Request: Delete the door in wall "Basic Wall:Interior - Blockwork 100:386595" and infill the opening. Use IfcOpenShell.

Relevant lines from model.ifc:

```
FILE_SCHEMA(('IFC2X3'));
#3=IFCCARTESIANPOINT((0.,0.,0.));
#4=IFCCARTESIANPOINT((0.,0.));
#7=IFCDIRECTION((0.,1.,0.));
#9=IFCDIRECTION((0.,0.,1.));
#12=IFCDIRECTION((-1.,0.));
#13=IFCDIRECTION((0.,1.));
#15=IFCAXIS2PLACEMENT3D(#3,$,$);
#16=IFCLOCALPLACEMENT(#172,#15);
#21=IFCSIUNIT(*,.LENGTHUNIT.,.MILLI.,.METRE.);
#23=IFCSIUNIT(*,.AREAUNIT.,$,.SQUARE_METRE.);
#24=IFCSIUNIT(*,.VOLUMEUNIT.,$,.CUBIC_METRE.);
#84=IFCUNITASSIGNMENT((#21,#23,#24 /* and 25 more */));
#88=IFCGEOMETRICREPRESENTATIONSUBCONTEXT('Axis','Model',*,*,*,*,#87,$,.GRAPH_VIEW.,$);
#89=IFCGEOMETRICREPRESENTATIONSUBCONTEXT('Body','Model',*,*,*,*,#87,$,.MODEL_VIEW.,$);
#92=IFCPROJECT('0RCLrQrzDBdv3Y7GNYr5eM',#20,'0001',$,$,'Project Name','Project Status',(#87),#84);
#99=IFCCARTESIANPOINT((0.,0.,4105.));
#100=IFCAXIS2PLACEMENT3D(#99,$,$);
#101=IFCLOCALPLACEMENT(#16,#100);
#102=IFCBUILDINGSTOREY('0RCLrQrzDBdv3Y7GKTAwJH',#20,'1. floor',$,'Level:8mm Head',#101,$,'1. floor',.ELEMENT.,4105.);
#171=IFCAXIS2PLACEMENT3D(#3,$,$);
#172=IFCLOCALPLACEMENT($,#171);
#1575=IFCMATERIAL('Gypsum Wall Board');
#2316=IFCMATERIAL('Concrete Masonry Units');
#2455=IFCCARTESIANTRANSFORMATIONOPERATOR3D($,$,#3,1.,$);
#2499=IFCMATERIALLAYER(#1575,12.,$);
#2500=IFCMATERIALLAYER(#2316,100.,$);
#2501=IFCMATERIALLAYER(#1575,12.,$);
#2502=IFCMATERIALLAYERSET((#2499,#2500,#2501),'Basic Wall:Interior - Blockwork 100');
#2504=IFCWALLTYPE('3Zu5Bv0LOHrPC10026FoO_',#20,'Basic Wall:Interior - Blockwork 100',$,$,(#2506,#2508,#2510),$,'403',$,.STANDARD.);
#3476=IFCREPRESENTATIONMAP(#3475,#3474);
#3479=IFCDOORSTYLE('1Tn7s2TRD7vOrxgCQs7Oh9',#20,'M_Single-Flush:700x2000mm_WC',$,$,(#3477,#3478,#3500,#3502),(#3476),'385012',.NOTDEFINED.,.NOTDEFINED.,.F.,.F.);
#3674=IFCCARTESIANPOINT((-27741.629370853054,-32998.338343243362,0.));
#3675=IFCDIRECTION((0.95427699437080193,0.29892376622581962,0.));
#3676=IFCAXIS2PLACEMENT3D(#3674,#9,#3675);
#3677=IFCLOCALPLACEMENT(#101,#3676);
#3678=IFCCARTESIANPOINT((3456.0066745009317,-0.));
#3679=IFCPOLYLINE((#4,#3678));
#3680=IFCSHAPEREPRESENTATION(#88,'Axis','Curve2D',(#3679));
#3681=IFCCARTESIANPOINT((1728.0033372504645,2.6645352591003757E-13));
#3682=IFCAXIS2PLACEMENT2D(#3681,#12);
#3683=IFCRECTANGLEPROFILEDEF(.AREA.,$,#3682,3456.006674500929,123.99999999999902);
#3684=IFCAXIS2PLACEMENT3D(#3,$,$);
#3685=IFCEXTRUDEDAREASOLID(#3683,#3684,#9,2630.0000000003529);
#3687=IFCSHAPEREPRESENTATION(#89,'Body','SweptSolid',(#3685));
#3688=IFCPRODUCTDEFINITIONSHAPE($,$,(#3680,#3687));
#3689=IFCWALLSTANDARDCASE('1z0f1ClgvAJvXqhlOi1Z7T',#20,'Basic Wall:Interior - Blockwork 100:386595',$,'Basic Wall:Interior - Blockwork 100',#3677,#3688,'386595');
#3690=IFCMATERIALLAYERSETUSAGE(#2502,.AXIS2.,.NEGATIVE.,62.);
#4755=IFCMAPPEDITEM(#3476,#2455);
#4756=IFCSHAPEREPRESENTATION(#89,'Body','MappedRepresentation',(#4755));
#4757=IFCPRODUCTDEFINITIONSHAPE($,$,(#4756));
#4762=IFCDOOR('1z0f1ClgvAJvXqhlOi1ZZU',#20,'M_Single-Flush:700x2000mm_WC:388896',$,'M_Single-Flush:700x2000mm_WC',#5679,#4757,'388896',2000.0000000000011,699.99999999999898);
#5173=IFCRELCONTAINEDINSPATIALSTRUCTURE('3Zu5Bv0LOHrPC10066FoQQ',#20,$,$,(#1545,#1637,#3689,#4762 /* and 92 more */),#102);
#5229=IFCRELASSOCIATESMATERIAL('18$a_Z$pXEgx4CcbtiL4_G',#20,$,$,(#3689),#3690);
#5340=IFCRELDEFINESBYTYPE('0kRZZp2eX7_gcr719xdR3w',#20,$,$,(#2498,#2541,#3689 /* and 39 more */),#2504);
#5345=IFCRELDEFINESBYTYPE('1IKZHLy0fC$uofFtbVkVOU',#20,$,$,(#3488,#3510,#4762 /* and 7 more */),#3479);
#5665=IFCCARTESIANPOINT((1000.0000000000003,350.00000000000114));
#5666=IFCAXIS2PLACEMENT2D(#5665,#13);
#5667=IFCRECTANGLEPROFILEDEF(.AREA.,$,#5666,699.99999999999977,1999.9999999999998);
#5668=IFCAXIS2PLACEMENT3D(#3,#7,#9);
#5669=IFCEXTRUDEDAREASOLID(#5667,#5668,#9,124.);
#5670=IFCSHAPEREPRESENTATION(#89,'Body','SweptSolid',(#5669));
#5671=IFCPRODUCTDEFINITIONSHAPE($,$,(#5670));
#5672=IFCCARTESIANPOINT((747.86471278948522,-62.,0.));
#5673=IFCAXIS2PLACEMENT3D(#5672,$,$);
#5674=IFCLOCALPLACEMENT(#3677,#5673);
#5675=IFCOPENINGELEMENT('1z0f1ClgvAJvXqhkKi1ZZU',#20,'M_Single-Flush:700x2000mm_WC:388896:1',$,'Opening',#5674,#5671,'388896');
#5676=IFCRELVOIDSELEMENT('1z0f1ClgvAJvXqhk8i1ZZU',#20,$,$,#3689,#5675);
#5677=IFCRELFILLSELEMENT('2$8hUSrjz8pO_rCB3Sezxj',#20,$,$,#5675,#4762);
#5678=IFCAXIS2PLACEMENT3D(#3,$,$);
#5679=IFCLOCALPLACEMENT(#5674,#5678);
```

```python
import ifcopenshell
import ifcopenshell.api.feature
import ifcopenshell.api.root
import ifcopenshell.geom
import ifcopenshell.util.shape

model = ifcopenshell.open("model.ifc")
settings = ifcopenshell.geom.settings()


def volume(element):
    """Net volume in cubic metres, openings subtracted."""
    shape = ifcopenshell.geom.create_shape(settings, element)
    return ifcopenshell.util.shape.get_volume(shape.geometry)


door = model.by_id(4762)
opening = door.FillsVoids[0].RelatingOpeningElement
wall = opening.VoidsElements[0].RelatingBuildingElement
before = volume(wall)

ifcopenshell.api.root.remove_product(model, product=door)
ifcopenshell.api.feature.remove_feature(model, feature=opening)

after = volume(wall)

print(f"wall volume {before:.3f} -> {after:.3f} m3")

model.write("model_updated.ifc")
```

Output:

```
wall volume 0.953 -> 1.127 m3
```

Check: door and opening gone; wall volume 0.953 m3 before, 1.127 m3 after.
